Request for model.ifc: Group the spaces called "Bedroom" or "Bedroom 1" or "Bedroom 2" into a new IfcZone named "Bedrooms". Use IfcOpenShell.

First a look at what the model holds.

```python
import ifcopenshell

model = ifcopenshell.open("model.ifc")
print(model.schema)
seen = {}
for space in model.by_type("IfcSpace"):
    seen[space.LongName] = seen.get(space.LongName, 0) + 1
for name, count in sorted(seen.items(), key=str):
    print(count, "x", name)
print("zones:", [z.Name for z in model.by_type("IfcZone")][:20])
```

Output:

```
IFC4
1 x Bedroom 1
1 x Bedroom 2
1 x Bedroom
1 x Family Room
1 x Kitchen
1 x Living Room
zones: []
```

```python
import ifcopenshell
import ifcopenshell.api.group
import ifcopenshell.api.root

model = ifcopenshell.open("model.ifc")

names = {"Bedroom", "Bedroom 1", "Bedroom 2"}
spaces = [s for s in model.by_type("IfcSpace") if s.LongName in names]

zone = ifcopenshell.api.root.create_entity(model, ifc_class="IfcZone", name="Bedrooms")
ifcopenshell.api.group.assign_group(model, products=spaces, group=zone)
print(len(spaces), "spaces in", zone.Name)

model.write("model_updated.ifc")
```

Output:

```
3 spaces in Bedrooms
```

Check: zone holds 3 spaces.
